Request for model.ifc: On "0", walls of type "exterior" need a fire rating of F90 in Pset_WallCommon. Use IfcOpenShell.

First a look at what the model holds.

```python
import ifcopenshell
import ifcopenshell.util.element

model = ifcopenshell.open("model.ifc")
print(model.schema)
storey = next(s for s in model.by_type("IfcBuildingStorey") if s.Name == "0")
walls = [e for e in ifcopenshell.util.element.get_decomposition(storey) if e.is_a("IfcWall")]
seen = {}
for e in walls:
    element_type = ifcopenshell.util.element.get_type(e)
    key = (element_type.Name if element_type != e and element_type else None, ifcopenshell.util.element.get_pset(e, "Pset_WallCommon", "FireRating"))
    seen[key] = seen.get(key, 0) + 1
for (name, value), count in sorted(seen.items(), key=str):
    print(count, "x", name, "|", value)
```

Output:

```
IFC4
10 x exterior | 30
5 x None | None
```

```python
import ifcopenshell
import ifcopenshell.api.pset
import ifcopenshell.util.element

model = ifcopenshell.open("model.ifc")

storey = next(s for s in model.by_type("IfcBuildingStorey") if s.Name == "0")
walls = [e for e in ifcopenshell.util.element.get_decomposition(storey) if e.is_a("IfcWall")]

count = 0
for e in walls:
    element_type = ifcopenshell.util.element.get_type(e)
    if element_type in (None, e) or element_type.Name != "exterior":
        continue
    # add_pset returns the element's existing set when there is one.
    pset = ifcopenshell.api.pset.add_pset(model, product=e, name="Pset_WallCommon")
    ifcopenshell.api.pset.edit_pset(model, pset=pset, properties={"FireRating": "F90"})
    count += 1

print(count, "walls updated")

model.write("model_updated.ifc")
```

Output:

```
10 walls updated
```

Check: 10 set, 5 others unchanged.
